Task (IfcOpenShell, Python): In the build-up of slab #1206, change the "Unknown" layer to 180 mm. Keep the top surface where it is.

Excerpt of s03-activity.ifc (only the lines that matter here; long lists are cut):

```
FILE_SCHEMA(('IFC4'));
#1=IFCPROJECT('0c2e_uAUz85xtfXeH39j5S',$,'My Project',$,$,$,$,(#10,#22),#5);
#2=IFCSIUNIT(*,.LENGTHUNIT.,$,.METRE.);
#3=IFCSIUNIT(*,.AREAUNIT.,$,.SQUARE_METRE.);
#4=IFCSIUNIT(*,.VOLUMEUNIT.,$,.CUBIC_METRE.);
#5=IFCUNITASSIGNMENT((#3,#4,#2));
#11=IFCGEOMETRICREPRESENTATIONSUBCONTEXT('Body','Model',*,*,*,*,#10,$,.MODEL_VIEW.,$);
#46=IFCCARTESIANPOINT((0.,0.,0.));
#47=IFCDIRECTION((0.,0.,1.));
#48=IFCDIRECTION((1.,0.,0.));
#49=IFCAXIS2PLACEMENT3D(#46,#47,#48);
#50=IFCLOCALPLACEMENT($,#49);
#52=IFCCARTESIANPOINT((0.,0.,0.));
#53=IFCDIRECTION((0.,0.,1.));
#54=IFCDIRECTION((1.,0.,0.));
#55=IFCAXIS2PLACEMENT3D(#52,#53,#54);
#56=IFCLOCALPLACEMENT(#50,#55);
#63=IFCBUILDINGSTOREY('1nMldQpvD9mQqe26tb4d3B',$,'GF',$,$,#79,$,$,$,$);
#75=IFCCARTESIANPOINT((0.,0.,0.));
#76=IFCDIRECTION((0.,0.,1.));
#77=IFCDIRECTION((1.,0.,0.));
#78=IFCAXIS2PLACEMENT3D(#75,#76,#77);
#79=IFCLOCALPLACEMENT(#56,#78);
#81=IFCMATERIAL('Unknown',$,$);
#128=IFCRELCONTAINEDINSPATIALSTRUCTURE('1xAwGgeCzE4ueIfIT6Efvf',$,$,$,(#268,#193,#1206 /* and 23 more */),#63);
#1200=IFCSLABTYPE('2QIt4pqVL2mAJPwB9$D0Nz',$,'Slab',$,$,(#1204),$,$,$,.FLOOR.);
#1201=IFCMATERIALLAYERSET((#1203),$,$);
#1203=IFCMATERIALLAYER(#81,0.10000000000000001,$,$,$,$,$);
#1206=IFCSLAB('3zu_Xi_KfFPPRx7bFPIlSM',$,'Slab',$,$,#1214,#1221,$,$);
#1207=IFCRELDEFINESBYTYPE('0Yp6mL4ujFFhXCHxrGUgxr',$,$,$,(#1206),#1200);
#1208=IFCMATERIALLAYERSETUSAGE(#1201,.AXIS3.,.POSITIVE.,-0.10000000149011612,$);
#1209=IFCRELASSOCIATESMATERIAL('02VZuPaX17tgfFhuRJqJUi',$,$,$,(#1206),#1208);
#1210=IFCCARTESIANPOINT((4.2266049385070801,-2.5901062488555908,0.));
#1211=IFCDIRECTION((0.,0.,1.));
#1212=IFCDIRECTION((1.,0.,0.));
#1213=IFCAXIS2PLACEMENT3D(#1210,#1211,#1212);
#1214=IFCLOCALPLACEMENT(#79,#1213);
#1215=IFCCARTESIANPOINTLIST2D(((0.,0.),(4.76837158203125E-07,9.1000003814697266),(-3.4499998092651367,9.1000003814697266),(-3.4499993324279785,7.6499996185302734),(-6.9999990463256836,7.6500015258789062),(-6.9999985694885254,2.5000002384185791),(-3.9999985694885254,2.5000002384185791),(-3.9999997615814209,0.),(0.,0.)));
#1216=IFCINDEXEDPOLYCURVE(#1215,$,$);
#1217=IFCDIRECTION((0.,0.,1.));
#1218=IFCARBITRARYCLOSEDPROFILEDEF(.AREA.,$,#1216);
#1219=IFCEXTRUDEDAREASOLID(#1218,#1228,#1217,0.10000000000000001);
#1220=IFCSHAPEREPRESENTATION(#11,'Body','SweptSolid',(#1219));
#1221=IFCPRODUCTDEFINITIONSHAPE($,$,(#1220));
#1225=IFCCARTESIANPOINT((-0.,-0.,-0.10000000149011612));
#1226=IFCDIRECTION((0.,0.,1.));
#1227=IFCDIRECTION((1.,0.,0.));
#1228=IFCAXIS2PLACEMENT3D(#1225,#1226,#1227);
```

```python
import ifcopenshell
import ifcopenshell.util.element
import ifcopenshell.util.representation

model = ifcopenshell.open("s03-activity.ifc")

layer_set = model.by_id(1201)
layer = next(l for l in layer_set.MaterialLayers if l.Material and l.Material.Name == "Unknown")
change = 0.18 - layer.LayerThickness
layer.LayerThickness += change

# Geometry does not follow the layer set by itself.
slabs = [e for e in ifcopenshell.util.element.get_elements_by_material(model, layer_set) if e.is_a("IfcSlab")]
for slab in sorted(slabs, key=lambda e: e.id()):
    body = ifcopenshell.util.representation.get_representation(slab, "Model", "Body")
    solid = body.Items[0]
    old_depth = solid.Depth
    solid.Depth += change
    # Extruded upwards: lower the start of the extrusion so the top stays.
    x, y, z = solid.Position.Location.Coordinates
    solid.Position.Location = model.createIfcCartesianPoint((x, y, z - change))
    print(slab.id(), f"{old_depth:g} -> {solid.Depth:g}")

# The layers are counted up from the underside, which has moved.
for usage in {ifcopenshell.util.element.get_material(slab) for slab in slabs}:
    usage.OffsetFromReferenceLine -= change

model.write("s03-activity_updated.ifc")
```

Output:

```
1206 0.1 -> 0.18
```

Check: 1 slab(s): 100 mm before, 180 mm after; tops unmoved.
